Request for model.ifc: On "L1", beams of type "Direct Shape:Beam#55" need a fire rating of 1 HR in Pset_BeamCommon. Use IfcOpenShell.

First a look at what the model holds.

```python
import ifcopenshell
import ifcopenshell.util.element

model = ifcopenshell.open("model.ifc")
print(model.schema)
storey = next(s for s in model.by_type("IfcBuildingStorey") if s.Name == "L1")
beams = [e for e in ifcopenshell.util.element.get_decomposition(storey) if e.is_a("IfcBeam")]
seen = {}
for e in beams:
    element_type = ifcopenshell.util.element.get_type(e)
    key = (element_type.Name if element_type != e and element_type else None, ifcopenshell.util.element.get_pset(e, "Pset_BeamCommon", "FireRating"))
    seen[key] = seen.get(key, 0) + 1
for (name, value), count in sorted(seen.items(), key=str):
    print(count, "x", name, "|", value)
```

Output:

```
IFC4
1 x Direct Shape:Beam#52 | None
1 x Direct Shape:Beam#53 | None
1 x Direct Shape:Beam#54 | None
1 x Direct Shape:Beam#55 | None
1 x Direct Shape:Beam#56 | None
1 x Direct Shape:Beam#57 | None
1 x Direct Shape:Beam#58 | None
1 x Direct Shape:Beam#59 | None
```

```python
import ifcopenshell
import ifcopenshell.api.pset
import ifcopenshell.util.element

model = ifcopenshell.open("model.ifc")

storey = next(s for s in model.by_type("IfcBuildingStorey") if s.Name == "L1")
beams = [e for e in ifcopenshell.util.element.get_decomposition(storey) if e.is_a("IfcBeam")]

count = 0
for e in beams:
    element_type = ifcopenshell.util.element.get_type(e)
    if element_type in (None, e) or element_type.Name != "Direct Shape:Beam#55":
        continue
    # add_pset returns the element's existing set when there is one.
    pset = ifcopenshell.api.pset.add_pset(model, product=e, name="Pset_BeamCommon")
    ifcopenshell.api.pset.edit_pset(model, pset=pset, properties={"FireRating": "1 HR"})
    count += 1

print(count, "beams updated")

model.write("model_edited.ifc")
```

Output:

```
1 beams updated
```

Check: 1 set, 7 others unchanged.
